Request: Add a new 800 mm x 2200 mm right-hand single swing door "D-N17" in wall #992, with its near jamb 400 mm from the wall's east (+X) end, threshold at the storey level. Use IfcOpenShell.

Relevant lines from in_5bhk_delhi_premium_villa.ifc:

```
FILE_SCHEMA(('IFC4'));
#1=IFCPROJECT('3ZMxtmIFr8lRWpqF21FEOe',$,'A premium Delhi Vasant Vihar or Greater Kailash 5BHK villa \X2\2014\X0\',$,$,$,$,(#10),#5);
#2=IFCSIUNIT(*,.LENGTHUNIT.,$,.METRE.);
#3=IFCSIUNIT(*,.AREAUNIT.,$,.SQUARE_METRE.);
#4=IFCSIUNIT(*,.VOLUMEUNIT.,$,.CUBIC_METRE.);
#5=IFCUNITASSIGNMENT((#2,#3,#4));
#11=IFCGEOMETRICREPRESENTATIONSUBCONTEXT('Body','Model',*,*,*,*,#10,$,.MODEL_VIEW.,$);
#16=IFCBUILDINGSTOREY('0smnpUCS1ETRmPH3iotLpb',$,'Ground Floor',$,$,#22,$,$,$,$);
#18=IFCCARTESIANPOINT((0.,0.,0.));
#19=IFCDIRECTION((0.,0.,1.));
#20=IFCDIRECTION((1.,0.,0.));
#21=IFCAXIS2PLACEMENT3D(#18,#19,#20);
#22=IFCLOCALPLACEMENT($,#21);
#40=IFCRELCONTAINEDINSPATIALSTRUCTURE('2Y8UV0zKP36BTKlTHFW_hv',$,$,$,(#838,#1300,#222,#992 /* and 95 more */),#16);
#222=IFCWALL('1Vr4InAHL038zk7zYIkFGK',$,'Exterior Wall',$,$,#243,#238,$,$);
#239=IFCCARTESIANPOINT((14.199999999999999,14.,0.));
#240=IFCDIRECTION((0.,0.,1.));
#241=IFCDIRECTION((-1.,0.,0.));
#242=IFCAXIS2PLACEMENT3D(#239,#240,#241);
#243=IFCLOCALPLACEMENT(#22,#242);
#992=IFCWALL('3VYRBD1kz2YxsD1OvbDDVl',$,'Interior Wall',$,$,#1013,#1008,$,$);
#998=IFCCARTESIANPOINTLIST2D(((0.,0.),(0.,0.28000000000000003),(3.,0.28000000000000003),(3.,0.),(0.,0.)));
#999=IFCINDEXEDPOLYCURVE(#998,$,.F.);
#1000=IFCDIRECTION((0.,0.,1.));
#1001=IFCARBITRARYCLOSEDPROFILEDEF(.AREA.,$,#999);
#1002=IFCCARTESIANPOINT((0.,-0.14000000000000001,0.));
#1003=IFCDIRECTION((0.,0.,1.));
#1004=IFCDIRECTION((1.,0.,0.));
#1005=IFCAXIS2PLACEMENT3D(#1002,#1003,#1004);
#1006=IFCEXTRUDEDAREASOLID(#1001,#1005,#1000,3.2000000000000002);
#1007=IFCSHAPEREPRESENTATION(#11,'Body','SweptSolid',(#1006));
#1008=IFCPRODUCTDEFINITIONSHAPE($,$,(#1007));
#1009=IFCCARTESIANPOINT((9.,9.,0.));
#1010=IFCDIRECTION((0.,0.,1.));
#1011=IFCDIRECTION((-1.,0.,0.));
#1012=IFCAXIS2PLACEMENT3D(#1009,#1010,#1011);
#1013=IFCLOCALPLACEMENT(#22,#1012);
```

```python
import numpy as np
import ifcopenshell
import ifcopenshell.api.feature
import ifcopenshell.api.geometry
import ifcopenshell.api.root
import ifcopenshell.api.spatial
import ifcopenshell.geom
import ifcopenshell.util.element
import ifcopenshell.util.placement
import ifcopenshell.util.representation
import ifcopenshell.util.shape
import ifcopenshell.util.unit

model = ifcopenshell.open("in_5bhk_delhi_premium_villa.ifc")
unit_scale = ifcopenshell.util.unit.calculate_unit_scale(model)
settings = ifcopenshell.geom.settings()


def volume(element):
    """Net volume in cubic metres, openings subtracted."""
    shape = ifcopenshell.geom.create_shape(settings, element)
    return ifcopenshell.util.shape.get_volume(shape.geometry)


wall = model.by_id(992)
storey = ifcopenshell.util.element.get_container(wall, ifc_class="IfcBuildingStorey")
context = ifcopenshell.util.representation.get_context(model, "Model", "Body", "MODEL_VIEW")
before = volume(wall)

width, height, from_end, sill = 0.8, 2.2, 0.4, 0.0  # metres

# The wall runs along its own X axis, and the end named is its -X end.
wall_shape = ifcopenshell.geom.create_shape(settings, wall)
x, y, z = ifcopenshell.util.shape.get_vertices(wall_shape.geometry).T
start = x.min() + from_end
face, thickness = float(y.min()), float(y.max() - y.min())
wall_matrix = ifcopenshell.util.placement.get_local_placement(wall.ObjectPlacement)
level = ifcopenshell.util.placement.get_local_placement(storey.ObjectPlacement)[2, 3]


def in_wall(x, y):
    """Placement at x, y metres in the wall's axes, at sill height."""
    matrix = wall_matrix.copy()
    matrix[:, 3] = wall_matrix @ np.array([x / unit_scale, y / unit_scale, 0.0, 1.0])
    matrix[2, 3] = level + sill / unit_scale
    return matrix


# Opening: a box that overshoots both wall faces by 50 mm.
opening = ifcopenshell.api.root.create_entity(model, ifc_class="IfcOpeningElement", predefined_type="OPENING")
box = ifcopenshell.api.geometry.add_wall_representation(
    model, context=context, length=width, height=height, thickness=thickness + 0.1
)
ifcopenshell.api.geometry.assign_representation(model, product=opening, representation=box)
ifcopenshell.api.geometry.edit_object_placement(model, product=opening, matrix=in_wall(start, face - 0.05), is_si=False)
ifcopenshell.api.feature.add_feature(model, feature=opening, element=wall)

door = ifcopenshell.api.root.create_entity(model, ifc_class="IfcDoor", name="D-N17", predefined_type="DOOR")
door.OverallWidth, door.OverallHeight = width / unit_scale, height / unit_scale
door.OperationType = "SINGLE_SWING_RIGHT"
body = ifcopenshell.api.geometry.add_door_representation(
    model,
    context=context,
    overall_width=door.OverallWidth,
    overall_height=door.OverallHeight,
    operation_type="SINGLE_SWING_RIGHT",
    lining_properties={"LiningDepth": thickness / unit_scale, "ThresholdDepth": thickness / unit_scale},
)
ifcopenshell.api.geometry.assign_representation(model, product=door, representation=body)
ifcopenshell.api.spatial.assign_container(model, products=[door], relating_structure=storey)
ifcopenshell.api.feature.add_filling(model, opening=opening, element=door)

# The lining spans the wall, so the door starts at the wall face.
ifcopenshell.api.geometry.edit_object_placement(model, product=door, matrix=in_wall(start, face), is_si=False)

after = volume(wall)

print(f"wall volume {before:.3f} -> {after:.3f} m3")

model.write("in_5bhk_delhi_premium_villa_rev.ifc")
```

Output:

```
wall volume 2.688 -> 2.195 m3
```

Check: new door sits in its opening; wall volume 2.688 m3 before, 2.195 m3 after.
